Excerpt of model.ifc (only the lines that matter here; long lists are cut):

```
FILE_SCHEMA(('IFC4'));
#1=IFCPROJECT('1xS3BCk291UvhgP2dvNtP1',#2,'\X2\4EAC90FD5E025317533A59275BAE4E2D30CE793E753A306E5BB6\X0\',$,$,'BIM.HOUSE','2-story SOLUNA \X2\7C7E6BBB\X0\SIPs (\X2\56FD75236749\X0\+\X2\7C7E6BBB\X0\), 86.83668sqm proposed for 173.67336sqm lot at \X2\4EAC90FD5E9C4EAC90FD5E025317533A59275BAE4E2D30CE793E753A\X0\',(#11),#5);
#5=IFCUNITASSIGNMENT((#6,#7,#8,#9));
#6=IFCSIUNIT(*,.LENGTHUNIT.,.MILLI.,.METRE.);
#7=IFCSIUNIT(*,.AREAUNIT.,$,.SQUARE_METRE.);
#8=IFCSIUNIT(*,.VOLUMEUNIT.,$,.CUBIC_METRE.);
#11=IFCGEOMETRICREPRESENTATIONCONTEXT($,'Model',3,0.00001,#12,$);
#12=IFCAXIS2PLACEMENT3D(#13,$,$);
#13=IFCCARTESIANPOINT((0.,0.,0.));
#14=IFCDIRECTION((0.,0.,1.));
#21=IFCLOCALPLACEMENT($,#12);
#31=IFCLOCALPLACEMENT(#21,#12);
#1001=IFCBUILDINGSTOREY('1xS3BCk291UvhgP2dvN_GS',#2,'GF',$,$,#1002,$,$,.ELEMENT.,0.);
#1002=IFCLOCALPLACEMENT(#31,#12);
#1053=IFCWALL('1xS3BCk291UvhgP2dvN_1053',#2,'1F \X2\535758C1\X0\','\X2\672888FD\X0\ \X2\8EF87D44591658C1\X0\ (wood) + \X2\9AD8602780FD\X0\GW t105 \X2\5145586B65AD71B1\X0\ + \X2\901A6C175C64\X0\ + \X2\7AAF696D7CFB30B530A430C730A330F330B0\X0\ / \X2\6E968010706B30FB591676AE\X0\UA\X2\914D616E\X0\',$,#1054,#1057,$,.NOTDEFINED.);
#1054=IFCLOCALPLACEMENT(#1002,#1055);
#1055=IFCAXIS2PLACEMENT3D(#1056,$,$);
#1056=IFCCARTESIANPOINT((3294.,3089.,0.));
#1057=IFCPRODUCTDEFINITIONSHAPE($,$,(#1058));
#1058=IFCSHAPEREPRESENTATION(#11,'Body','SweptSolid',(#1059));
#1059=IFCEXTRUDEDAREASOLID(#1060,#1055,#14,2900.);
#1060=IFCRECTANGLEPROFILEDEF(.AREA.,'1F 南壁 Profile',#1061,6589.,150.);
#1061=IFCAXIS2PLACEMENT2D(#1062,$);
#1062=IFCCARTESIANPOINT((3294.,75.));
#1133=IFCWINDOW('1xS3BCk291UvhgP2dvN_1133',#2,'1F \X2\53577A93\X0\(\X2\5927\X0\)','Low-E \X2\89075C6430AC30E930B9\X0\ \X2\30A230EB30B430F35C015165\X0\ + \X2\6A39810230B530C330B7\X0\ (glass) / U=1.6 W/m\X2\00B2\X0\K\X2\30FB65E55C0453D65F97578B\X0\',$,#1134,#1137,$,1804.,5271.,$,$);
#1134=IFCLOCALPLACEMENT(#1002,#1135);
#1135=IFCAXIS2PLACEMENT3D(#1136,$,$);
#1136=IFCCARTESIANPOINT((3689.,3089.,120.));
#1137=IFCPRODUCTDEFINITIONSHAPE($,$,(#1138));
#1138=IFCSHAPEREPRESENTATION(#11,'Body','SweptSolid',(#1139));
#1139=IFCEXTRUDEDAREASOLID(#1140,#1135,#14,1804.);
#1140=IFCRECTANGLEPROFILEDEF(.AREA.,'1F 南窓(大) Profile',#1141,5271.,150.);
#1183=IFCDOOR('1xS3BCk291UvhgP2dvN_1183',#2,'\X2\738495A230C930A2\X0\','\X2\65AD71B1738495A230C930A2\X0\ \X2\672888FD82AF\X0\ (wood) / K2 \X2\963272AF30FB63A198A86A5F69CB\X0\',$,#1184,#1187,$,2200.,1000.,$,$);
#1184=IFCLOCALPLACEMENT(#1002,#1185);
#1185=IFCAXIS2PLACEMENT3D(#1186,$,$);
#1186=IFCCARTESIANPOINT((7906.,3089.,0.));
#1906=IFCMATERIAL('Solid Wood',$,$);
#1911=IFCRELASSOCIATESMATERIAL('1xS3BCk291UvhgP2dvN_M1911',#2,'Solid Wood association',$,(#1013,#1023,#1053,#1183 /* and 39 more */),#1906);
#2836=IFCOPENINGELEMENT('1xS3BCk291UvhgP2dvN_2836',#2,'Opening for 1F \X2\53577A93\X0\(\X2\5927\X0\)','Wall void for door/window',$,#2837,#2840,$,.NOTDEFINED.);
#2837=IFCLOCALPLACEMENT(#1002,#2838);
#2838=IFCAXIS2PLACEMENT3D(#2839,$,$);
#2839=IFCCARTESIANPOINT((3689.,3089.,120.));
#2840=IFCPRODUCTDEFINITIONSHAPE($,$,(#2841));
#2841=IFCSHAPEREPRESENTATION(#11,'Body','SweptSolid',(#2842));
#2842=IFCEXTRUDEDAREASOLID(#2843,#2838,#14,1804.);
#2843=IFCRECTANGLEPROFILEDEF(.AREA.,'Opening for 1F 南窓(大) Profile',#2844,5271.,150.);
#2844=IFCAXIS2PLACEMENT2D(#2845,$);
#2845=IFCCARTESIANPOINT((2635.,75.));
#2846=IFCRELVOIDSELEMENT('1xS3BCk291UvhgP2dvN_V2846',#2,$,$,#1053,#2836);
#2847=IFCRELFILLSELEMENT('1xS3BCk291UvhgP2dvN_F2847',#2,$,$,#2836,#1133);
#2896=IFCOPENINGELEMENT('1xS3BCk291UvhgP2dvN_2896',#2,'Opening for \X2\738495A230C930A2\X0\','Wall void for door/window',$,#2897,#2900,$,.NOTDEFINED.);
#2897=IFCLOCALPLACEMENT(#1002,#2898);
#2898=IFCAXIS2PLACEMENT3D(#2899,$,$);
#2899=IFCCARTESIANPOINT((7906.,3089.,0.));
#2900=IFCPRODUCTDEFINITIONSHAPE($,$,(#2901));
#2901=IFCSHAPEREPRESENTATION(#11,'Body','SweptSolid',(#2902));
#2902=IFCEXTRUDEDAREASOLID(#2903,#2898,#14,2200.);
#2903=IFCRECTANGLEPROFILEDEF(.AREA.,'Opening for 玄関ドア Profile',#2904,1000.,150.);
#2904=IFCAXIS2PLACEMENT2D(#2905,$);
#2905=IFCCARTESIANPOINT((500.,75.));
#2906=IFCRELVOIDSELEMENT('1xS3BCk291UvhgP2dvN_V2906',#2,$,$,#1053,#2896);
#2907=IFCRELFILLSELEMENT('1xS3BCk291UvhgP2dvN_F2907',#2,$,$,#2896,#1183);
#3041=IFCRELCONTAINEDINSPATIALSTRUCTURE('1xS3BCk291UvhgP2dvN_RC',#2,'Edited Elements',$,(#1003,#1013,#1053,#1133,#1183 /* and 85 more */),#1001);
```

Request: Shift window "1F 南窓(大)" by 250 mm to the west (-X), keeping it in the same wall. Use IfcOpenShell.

```python
import ifcopenshell
import ifcopenshell.api.geometry
import ifcopenshell.util.placement

model = ifcopenshell.open("model.ifc")

window = model.by_guid("1xS3BCk291UvhgP2dvN_1133")
opening = window.FillsVoids[0].RelatingOpeningElement
wall = opening.VoidsElements[0].RelatingBuildingElement

wall_matrix = ifcopenshell.util.placement.get_local_placement(wall.ObjectPlacement)
shift = wall_matrix[:3, 0] * -250.0
before = ifcopenshell.util.placement.get_local_placement(window.ObjectPlacement)[:3, 3].copy()

# The window is not placed relative to its opening, so move both.
for product in (opening, window):
    matrix = ifcopenshell.util.placement.get_local_placement(product.ObjectPlacement)
    matrix[:3, 3] += shift
    ifcopenshell.api.geometry.edit_object_placement(model, product=product, matrix=matrix, is_si=False)

after = ifcopenshell.util.placement.get_local_placement(window.ObjectPlacement)[:3, 3]
print("window moved by", (after - before).round(3) + 0.0)

model.write("model-out.ifc")
```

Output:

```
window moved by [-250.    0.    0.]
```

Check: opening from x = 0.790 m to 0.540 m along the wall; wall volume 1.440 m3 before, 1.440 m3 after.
